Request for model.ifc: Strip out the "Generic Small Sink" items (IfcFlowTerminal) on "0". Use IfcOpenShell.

First a look at what the model holds.

```python
import ifcopenshell
import ifcopenshell.util.element

model = ifcopenshell.open("model.ifc")
print(model.schema)
storey = next(s for s in model.by_type("IfcBuildingStorey") if s.Name == "0")
terminals = [e for e in ifcopenshell.util.element.get_decomposition(storey) if e.is_a("IfcFlowTerminal")]
seen = {}
for e in terminals:
    element_type = ifcopenshell.util.element.get_type(e)
    name = element_type.Name if element_type not in (None, e) else None
    seen[name] = seen.get(name, 0) + 1
for name, count in sorted(seen.items(), key=str):
    print(count, "x", name)
```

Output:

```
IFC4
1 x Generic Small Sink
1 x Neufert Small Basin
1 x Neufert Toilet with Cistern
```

```python
import ifcopenshell
import ifcopenshell.api.root
import ifcopenshell.util.element

model = ifcopenshell.open("model.ifc")

storey = next(s for s in model.by_type("IfcBuildingStorey") if s.Name == "0")
terminals = [e for e in ifcopenshell.util.element.get_decomposition(storey) if e.is_a("IfcFlowTerminal")]
targets = [e for e in terminals if (t := ifcopenshell.util.element.get_type(e)) not in (None, e) and t.Name == "Generic Small Sink"]

for e in targets:
    ifcopenshell.api.root.remove_product(model, product=e)
print(len(targets), "removed")

model.write("model-out.ifc")
```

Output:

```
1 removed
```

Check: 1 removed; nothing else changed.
